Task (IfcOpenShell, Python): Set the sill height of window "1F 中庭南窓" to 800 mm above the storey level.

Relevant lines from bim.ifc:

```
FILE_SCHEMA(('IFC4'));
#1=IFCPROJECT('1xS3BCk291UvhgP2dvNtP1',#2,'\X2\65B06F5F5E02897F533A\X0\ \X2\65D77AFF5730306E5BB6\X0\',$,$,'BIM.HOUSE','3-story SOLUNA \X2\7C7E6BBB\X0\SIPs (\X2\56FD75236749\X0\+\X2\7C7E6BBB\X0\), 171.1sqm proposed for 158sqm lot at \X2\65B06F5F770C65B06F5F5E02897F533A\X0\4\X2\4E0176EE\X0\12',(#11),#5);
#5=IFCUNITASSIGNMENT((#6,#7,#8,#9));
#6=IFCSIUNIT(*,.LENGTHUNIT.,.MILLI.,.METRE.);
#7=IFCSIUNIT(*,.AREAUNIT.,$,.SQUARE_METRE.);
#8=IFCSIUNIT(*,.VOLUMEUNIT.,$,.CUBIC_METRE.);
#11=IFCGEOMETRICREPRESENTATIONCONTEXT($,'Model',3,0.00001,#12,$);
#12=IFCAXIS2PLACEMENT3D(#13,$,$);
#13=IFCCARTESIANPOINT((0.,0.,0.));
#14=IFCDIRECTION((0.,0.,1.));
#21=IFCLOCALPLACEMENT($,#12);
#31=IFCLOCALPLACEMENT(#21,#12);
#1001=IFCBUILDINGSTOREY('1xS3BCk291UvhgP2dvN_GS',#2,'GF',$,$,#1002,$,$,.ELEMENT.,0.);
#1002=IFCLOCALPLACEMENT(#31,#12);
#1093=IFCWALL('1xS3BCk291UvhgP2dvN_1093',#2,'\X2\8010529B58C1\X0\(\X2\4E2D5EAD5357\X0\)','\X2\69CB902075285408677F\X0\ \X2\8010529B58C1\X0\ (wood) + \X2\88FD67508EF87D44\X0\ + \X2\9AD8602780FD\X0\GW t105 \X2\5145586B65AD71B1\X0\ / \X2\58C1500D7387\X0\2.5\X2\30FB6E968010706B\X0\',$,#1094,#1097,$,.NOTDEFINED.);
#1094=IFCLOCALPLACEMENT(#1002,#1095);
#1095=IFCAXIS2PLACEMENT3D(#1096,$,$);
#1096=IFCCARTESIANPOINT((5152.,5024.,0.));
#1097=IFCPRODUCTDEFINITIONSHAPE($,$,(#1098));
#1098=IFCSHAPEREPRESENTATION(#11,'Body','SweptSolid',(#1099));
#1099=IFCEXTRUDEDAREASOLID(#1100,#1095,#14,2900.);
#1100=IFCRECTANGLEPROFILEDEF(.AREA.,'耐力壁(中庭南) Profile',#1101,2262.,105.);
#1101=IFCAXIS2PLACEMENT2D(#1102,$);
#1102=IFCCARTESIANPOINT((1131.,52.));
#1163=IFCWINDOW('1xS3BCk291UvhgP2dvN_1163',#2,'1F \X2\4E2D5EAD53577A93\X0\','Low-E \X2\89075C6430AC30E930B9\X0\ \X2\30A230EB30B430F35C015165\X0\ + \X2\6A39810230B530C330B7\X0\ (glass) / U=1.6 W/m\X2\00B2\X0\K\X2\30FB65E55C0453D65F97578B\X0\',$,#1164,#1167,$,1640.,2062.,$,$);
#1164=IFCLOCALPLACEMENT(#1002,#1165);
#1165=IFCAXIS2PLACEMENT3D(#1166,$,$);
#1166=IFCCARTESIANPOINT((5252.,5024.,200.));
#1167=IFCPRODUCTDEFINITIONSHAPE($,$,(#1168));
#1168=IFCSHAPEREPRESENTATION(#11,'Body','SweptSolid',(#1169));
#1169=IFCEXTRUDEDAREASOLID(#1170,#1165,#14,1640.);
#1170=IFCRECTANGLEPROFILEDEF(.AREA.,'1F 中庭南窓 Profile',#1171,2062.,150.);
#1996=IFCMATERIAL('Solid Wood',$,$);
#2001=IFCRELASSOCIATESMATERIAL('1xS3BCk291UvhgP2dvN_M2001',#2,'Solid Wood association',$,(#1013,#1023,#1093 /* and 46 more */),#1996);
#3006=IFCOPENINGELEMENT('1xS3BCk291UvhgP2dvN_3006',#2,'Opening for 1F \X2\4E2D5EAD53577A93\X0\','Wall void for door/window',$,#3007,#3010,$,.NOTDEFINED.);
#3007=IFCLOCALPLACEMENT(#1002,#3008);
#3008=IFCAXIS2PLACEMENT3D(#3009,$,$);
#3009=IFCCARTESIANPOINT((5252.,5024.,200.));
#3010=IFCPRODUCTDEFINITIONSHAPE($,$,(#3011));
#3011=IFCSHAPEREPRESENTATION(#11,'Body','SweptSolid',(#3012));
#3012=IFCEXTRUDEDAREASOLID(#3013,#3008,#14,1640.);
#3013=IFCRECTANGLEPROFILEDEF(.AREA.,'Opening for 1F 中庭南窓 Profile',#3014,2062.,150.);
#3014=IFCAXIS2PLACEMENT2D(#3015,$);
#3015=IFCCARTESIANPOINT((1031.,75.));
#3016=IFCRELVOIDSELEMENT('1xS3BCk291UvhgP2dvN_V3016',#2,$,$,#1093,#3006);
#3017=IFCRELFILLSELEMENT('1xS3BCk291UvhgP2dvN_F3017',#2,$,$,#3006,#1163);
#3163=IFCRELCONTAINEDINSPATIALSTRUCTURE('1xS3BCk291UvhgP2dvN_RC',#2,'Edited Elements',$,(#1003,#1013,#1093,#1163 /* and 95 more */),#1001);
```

```python
import numpy as np
import ifcopenshell
import ifcopenshell.api.geometry
import ifcopenshell.geom
import ifcopenshell.util.element
import ifcopenshell.util.placement
import ifcopenshell.util.shape
import ifcopenshell.util.unit

model = ifcopenshell.open("bim.ifc")
unit_scale = ifcopenshell.util.unit.calculate_unit_scale(model)

window = model.by_id(1163)
opening = window.FillsVoids[0].RelatingOpeningElement
storey = ifcopenshell.util.element.get_container(window, ifc_class="IfcBuildingStorey")
level = ifcopenshell.util.placement.get_local_placement(storey.ObjectPlacement)[2, 3]

# The opening's origin need not be at the sill, so measure its lowest point.
shape = ifcopenshell.geom.create_shape(ifcopenshell.geom.settings(), opening)
bottom = ifcopenshell.util.shape.get_shape_bottom_elevation(shape, shape.geometry) / unit_scale
dz = level + 800.0 - bottom

shift = np.array([0.0, 0.0, dz])
# The window is not placed relative to its opening, so move both.
for product in (opening, window):
    matrix = ifcopenshell.util.placement.get_local_placement(product.ObjectPlacement)
    matrix[:3, 3] += shift
    ifcopenshell.api.geometry.edit_object_placement(model, product=product, matrix=matrix, is_si=False)

print(f"moved by {dz * unit_scale:+.3f} m")

model.write("bim_rev.ifc")
```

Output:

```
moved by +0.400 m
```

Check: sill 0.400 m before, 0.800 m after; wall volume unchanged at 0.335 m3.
